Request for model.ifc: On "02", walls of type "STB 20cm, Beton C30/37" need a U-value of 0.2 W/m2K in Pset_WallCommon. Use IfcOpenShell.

First a look at what the model holds.

```python
import ifcopenshell
import ifcopenshell.util.element

model = ifcopenshell.open("model.ifc")
print(model.schema)
storey = next(s for s in model.by_type("IfcBuildingStorey") if s.Name == "02")
walls = [e for e in ifcopenshell.util.element.get_decomposition(storey) if e.is_a("IfcWall")]
seen = {}
for e in walls:
    element_type = ifcopenshell.util.element.get_type(e)
    key = (element_type.Name if element_type != e and element_type else None, ifcopenshell.util.element.get_pset(e, "Pset_WallCommon", "ThermalTransmittance"))
    seen[key] = seen.get(key, 0) + 1
for (name, value), count in sorted(seen.items(), key=str):
    print(count, "x", name, "|", value)
```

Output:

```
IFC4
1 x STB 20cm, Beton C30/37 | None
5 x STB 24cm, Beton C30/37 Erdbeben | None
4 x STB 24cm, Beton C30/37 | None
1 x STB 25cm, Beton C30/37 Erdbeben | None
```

```python
import ifcopenshell
import ifcopenshell.api.pset
import ifcopenshell.util.element

model = ifcopenshell.open("model.ifc")

storey = next(s for s in model.by_type("IfcBuildingStorey") if s.Name == "02")
walls = [e for e in ifcopenshell.util.element.get_decomposition(storey) if e.is_a("IfcWall")]

count = 0
for e in walls:
    element_type = ifcopenshell.util.element.get_type(e)
    if element_type in (None, e) or element_type.Name != "STB 20cm, Beton C30/37":
        continue
    # add_pset returns the element's existing set when there is one.
    pset = ifcopenshell.api.pset.add_pset(model, product=e, name="Pset_WallCommon")
    ifcopenshell.api.pset.edit_pset(model, pset=pset, properties={"ThermalTransmittance": 0.2})
    count += 1

print(count, "walls updated")

model.write("model_v2.ifc")
```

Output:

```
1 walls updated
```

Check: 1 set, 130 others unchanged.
